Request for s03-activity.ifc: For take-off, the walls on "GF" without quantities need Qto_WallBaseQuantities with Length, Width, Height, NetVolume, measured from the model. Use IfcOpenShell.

First a look at what the model holds.

```python
import ifcopenshell
import ifcopenshell.util.element
import ifcopenshell.util.unit

model = ifcopenshell.open("s03-activity.ifc")
print(model.schema)
for unit_type in ("LENGTHUNIT", "AREAUNIT", "VOLUMEUNIT"):
    print(unit_type, ifcopenshell.util.unit.calculate_unit_scale(model, unit_type))
storey = next(s for s in model.by_type("IfcBuildingStorey") if s.Name == "GF")
walls = [e for e in ifcopenshell.util.element.get_decomposition(storey) if e.is_a("IfcWall")]
for e in sorted(walls, key=lambda e: e.id()):
    print(e.id(), e.is_a(), e.Name, list(ifcopenshell.util.element.get_psets(e, qtos_only=True)), sep=" | ")
```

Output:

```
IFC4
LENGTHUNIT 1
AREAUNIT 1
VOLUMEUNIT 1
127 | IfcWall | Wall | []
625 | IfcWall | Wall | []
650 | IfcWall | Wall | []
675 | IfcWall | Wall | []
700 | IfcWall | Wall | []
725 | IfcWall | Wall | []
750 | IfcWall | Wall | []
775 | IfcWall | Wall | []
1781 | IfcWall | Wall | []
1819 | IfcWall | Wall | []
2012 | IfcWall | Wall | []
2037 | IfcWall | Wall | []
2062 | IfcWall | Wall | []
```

```python
import ifcopenshell
import ifcopenshell.api.pset
import ifcopenshell.geom
import ifcopenshell.util.element
import ifcopenshell.util.shape
import ifcopenshell.util.unit

model = ifcopenshell.open("s03-activity.ifc")
unit_scale = ifcopenshell.util.unit.calculate_unit_scale(model)
volume_scale = ifcopenshell.util.unit.calculate_unit_scale(model, "VOLUMEUNIT")
settings = ifcopenshell.geom.settings()

storey = next(s for s in model.by_type("IfcBuildingStorey") if s.Name == "GF")
walls = [e for e in ifcopenshell.util.element.get_decomposition(storey) if e.is_a("IfcWall")]

for e in sorted(walls, key=lambda e: e.id()):
    if ifcopenshell.util.element.get_psets(e, qtos_only=True, should_inherit=False):
        continue
    # Geometry comes back in metres, in the element's own axes.
    shape = ifcopenshell.geom.create_shape(settings, e)
    values = {
        "Length": ifcopenshell.util.shape.get_x(shape.geometry) / unit_scale,
        "Width": ifcopenshell.util.shape.get_y(shape.geometry) / unit_scale,
        "Height": ifcopenshell.util.shape.get_z(shape.geometry) / unit_scale,
        "NetVolume": ifcopenshell.util.shape.get_volume(shape.geometry) / volume_scale,
    }
    qto = ifcopenshell.api.pset.add_qto(model, product=e, name="Qto_WallBaseQuantities")
    ifcopenshell.api.pset.edit_qto(model, qto=qto, properties=values)
    print(e.id(), {k: round(v, 3) for k, v in values.items()})

model.write("s03-activity_edited.ifc")
```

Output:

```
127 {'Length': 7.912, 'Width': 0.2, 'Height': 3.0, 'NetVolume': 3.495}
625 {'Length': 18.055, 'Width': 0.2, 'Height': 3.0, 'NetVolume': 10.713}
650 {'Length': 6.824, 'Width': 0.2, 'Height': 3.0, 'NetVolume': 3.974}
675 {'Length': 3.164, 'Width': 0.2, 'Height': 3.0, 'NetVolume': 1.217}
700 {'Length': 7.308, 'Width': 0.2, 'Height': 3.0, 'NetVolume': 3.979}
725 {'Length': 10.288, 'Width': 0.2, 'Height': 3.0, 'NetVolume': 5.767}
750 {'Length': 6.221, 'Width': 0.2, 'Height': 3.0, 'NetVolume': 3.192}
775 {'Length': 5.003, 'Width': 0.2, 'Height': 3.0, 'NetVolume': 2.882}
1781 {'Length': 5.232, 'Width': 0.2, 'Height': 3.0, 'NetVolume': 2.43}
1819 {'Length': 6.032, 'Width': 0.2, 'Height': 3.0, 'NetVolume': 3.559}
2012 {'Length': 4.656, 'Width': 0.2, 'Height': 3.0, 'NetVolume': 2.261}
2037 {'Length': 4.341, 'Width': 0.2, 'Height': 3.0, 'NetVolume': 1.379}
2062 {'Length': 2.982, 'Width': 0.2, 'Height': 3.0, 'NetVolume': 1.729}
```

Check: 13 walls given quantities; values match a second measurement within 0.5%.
